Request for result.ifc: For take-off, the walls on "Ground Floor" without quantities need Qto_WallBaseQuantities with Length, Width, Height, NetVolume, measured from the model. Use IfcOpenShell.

First a look at what the model holds.

```python
import ifcopenshell
import ifcopenshell.util.element
import ifcopenshell.util.unit

model = ifcopenshell.open("result.ifc")
print(model.schema)
for unit_type in ("LENGTHUNIT", "AREAUNIT", "VOLUMEUNIT"):
    print(unit_type, ifcopenshell.util.unit.calculate_unit_scale(model, unit_type))
storey = next(s for s in model.by_type("IfcBuildingStorey") if s.Name == "Ground Floor")
walls = [e for e in ifcopenshell.util.element.get_decomposition(storey) if e.is_a("IfcWall")]
for e in sorted(walls, key=lambda e: e.id()):
    print(e.id(), e.is_a(), e.Name, list(ifcopenshell.util.element.get_psets(e, qtos_only=True)), sep=" | ")
```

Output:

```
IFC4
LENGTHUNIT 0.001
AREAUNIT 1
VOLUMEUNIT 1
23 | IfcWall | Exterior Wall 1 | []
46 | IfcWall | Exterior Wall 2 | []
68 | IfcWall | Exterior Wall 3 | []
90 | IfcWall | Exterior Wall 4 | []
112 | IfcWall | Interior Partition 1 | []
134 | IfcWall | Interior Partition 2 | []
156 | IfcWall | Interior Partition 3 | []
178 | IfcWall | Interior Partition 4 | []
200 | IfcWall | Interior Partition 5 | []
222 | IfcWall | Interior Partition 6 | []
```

```python
import ifcopenshell
import ifcopenshell.api.pset
import ifcopenshell.geom
import ifcopenshell.util.element
import ifcopenshell.util.shape
import ifcopenshell.util.unit

model = ifcopenshell.open("result.ifc")
unit_scale = ifcopenshell.util.unit.calculate_unit_scale(model)
volume_scale = ifcopenshell.util.unit.calculate_unit_scale(model, "VOLUMEUNIT")
settings = ifcopenshell.geom.settings()

storey = next(s for s in model.by_type("IfcBuildingStorey") if s.Name == "Ground Floor")
walls = [e for e in ifcopenshell.util.element.get_decomposition(storey) if e.is_a("IfcWall")]

for e in sorted(walls, key=lambda e: e.id()):
    if ifcopenshell.util.element.get_psets(e, qtos_only=True, should_inherit=False):
        continue
    # Geometry comes back in metres, in the element's own axes.
    shape = ifcopenshell.geom.create_shape(settings, e)
    values = {
        "Length": ifcopenshell.util.shape.get_x(shape.geometry) / unit_scale,
        "Width": ifcopenshell.util.shape.get_y(shape.geometry) / unit_scale,
        "Height": ifcopenshell.util.shape.get_z(shape.geometry) / unit_scale,
        "NetVolume": ifcopenshell.util.shape.get_volume(shape.geometry) / volume_scale,
    }
    qto = ifcopenshell.api.pset.add_qto(model, product=e, name="Qto_WallBaseQuantities")
    ifcopenshell.api.pset.edit_qto(model, qto=qto, properties=values)
    print(e.id(), {k: round(v, 3) for k, v in values.items()})

model.write("result_rev.ifc")
```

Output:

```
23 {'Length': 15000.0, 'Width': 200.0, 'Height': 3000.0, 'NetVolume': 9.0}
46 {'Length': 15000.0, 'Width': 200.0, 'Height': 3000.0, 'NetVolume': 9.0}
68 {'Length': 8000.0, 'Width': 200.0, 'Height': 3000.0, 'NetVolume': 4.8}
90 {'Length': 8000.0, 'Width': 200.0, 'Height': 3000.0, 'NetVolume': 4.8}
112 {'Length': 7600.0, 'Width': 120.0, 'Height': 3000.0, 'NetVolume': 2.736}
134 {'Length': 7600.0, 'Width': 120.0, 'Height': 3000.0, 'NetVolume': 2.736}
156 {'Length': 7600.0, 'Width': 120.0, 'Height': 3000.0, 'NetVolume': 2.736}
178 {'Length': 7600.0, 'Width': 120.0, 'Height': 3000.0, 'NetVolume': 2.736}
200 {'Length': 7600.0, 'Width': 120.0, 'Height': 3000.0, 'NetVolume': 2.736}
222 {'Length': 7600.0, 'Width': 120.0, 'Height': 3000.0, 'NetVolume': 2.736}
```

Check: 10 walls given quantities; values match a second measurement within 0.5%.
